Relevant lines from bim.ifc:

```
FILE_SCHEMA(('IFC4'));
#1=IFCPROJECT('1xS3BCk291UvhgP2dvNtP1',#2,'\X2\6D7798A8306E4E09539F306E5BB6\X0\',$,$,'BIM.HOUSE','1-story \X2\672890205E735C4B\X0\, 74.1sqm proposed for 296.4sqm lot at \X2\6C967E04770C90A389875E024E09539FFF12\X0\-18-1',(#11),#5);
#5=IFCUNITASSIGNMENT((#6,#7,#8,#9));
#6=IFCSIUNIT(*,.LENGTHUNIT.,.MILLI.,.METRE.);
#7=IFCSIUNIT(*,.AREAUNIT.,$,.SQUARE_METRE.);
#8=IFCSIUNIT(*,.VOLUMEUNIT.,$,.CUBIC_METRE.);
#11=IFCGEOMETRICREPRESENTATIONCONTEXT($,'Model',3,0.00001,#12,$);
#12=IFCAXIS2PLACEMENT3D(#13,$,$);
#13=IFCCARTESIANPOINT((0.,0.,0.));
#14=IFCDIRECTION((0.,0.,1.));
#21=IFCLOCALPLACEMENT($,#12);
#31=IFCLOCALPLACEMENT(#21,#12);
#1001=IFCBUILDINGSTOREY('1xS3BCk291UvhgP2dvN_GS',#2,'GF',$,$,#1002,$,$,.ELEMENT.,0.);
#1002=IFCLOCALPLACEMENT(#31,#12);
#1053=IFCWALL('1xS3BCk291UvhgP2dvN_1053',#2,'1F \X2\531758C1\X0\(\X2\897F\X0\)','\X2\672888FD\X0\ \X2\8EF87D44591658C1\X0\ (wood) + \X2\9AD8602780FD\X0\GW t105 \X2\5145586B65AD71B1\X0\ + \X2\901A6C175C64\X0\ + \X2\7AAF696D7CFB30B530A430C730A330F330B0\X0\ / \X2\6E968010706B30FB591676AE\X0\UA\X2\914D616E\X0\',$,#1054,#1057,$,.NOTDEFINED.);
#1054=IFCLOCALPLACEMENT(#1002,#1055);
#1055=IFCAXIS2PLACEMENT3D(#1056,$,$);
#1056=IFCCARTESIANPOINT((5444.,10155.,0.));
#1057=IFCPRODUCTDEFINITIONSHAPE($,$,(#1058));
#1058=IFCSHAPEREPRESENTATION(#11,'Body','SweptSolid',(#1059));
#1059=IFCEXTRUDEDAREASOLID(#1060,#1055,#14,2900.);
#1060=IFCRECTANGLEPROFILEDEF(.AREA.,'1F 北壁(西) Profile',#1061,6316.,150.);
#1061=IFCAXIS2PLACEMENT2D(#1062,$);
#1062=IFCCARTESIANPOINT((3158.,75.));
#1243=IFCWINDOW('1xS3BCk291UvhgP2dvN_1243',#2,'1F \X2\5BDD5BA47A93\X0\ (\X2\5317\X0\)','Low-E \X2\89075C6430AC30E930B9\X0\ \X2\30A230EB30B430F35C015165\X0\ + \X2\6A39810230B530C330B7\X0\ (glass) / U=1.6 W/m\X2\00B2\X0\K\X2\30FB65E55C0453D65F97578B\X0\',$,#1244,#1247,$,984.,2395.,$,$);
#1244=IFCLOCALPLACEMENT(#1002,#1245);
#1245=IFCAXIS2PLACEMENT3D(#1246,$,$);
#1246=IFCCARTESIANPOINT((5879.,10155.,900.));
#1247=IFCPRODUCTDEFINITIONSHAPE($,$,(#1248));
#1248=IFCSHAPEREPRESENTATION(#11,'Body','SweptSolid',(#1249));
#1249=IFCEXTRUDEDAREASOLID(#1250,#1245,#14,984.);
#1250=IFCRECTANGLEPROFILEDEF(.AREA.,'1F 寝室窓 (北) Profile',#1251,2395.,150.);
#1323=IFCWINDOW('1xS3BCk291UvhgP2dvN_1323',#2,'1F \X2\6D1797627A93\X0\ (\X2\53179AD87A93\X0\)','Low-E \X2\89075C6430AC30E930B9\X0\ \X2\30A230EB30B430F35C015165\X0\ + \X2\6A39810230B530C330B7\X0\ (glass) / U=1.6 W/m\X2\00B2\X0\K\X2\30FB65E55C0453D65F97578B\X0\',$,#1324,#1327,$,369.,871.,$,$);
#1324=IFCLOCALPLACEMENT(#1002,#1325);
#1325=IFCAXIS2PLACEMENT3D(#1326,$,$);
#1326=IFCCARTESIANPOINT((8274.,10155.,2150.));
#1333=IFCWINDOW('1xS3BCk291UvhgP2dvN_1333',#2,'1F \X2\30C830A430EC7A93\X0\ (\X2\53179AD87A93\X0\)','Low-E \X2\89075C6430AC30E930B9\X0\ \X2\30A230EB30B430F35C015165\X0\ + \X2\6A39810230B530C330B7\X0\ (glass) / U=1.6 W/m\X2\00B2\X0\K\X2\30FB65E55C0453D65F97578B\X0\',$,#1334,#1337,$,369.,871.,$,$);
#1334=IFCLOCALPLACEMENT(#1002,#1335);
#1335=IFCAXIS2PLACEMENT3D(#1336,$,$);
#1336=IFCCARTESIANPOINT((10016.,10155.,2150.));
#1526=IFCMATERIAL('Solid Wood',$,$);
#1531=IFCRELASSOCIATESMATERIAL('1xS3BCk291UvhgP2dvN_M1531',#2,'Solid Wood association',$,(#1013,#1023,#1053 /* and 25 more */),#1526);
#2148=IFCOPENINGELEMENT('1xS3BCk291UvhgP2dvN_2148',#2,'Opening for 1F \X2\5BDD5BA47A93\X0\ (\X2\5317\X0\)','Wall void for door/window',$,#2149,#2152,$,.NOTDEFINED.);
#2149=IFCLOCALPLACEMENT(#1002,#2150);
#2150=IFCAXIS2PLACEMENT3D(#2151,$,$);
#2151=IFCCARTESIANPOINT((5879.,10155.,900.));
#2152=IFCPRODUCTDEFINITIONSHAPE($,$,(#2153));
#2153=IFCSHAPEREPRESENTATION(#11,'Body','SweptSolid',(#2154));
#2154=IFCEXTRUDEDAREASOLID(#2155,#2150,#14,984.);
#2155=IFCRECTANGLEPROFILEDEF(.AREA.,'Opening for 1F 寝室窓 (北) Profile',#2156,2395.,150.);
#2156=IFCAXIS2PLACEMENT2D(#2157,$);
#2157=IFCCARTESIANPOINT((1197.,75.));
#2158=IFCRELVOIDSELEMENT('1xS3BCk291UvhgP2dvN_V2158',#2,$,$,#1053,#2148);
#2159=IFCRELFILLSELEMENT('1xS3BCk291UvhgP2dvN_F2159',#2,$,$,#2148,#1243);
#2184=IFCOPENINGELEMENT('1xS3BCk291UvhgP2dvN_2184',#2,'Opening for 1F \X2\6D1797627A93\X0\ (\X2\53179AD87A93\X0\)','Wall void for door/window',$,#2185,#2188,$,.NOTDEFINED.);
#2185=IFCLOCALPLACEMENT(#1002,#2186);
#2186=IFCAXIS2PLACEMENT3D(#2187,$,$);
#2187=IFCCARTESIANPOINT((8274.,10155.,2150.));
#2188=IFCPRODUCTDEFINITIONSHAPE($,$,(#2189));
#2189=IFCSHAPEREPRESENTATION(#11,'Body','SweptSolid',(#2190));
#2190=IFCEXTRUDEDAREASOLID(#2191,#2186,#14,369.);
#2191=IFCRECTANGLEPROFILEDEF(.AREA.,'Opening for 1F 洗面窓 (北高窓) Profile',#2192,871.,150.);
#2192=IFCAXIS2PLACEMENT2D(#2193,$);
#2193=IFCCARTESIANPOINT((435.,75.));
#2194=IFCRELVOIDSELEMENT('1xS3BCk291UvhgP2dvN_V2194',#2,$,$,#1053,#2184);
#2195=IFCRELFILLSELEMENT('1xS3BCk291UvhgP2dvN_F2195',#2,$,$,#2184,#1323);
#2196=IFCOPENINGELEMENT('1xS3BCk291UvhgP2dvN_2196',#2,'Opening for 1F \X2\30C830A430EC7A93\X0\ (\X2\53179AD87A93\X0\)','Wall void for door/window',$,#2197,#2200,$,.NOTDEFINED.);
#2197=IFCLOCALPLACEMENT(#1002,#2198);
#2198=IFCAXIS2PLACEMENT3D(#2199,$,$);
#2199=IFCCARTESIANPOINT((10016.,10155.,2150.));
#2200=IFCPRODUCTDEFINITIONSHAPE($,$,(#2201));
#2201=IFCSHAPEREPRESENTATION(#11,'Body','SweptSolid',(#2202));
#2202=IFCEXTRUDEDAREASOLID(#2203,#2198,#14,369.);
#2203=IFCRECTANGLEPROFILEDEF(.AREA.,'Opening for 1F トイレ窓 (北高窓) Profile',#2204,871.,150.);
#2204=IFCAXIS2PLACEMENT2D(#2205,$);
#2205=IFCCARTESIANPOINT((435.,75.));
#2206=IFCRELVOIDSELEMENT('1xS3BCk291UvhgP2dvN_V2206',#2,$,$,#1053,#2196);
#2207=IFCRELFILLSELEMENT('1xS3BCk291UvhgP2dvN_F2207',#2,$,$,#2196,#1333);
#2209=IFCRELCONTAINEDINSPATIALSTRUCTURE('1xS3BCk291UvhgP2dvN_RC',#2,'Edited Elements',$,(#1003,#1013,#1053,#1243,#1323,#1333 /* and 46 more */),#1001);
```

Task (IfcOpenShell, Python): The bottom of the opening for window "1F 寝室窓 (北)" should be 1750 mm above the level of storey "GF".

```python
import numpy as np
import ifcopenshell
import ifcopenshell.api.geometry
import ifcopenshell.geom
import ifcopenshell.util.element
import ifcopenshell.util.placement
import ifcopenshell.util.shape
import ifcopenshell.util.unit

model = ifcopenshell.open("bim.ifc")
unit_scale = ifcopenshell.util.unit.calculate_unit_scale(model)

window = model.by_id(1243)
opening = window.FillsVoids[0].RelatingOpeningElement
storey = ifcopenshell.util.element.get_container(window, ifc_class="IfcBuildingStorey")
level = ifcopenshell.util.placement.get_local_placement(storey.ObjectPlacement)[2, 3]

# The opening's origin need not be at the sill, so measure its lowest point.
shape = ifcopenshell.geom.create_shape(ifcopenshell.geom.settings(), opening)
bottom = ifcopenshell.util.shape.get_shape_bottom_elevation(shape, shape.geometry) / unit_scale
dz = level + 1.75 / unit_scale - bottom

shift = np.array([0.0, 0.0, dz])
# The window is not placed relative to its opening, so move both.
for product in (opening, window):
    matrix = ifcopenshell.util.placement.get_local_placement(product.ObjectPlacement)
    matrix[:3, 3] += shift
    ifcopenshell.api.geometry.edit_object_placement(model, product=product, matrix=matrix, is_si=False)

print(f"moved by {dz * unit_scale:+.3f} m")

model.write("bim_v2.ifc")
```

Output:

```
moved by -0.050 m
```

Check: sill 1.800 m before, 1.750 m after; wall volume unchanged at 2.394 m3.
